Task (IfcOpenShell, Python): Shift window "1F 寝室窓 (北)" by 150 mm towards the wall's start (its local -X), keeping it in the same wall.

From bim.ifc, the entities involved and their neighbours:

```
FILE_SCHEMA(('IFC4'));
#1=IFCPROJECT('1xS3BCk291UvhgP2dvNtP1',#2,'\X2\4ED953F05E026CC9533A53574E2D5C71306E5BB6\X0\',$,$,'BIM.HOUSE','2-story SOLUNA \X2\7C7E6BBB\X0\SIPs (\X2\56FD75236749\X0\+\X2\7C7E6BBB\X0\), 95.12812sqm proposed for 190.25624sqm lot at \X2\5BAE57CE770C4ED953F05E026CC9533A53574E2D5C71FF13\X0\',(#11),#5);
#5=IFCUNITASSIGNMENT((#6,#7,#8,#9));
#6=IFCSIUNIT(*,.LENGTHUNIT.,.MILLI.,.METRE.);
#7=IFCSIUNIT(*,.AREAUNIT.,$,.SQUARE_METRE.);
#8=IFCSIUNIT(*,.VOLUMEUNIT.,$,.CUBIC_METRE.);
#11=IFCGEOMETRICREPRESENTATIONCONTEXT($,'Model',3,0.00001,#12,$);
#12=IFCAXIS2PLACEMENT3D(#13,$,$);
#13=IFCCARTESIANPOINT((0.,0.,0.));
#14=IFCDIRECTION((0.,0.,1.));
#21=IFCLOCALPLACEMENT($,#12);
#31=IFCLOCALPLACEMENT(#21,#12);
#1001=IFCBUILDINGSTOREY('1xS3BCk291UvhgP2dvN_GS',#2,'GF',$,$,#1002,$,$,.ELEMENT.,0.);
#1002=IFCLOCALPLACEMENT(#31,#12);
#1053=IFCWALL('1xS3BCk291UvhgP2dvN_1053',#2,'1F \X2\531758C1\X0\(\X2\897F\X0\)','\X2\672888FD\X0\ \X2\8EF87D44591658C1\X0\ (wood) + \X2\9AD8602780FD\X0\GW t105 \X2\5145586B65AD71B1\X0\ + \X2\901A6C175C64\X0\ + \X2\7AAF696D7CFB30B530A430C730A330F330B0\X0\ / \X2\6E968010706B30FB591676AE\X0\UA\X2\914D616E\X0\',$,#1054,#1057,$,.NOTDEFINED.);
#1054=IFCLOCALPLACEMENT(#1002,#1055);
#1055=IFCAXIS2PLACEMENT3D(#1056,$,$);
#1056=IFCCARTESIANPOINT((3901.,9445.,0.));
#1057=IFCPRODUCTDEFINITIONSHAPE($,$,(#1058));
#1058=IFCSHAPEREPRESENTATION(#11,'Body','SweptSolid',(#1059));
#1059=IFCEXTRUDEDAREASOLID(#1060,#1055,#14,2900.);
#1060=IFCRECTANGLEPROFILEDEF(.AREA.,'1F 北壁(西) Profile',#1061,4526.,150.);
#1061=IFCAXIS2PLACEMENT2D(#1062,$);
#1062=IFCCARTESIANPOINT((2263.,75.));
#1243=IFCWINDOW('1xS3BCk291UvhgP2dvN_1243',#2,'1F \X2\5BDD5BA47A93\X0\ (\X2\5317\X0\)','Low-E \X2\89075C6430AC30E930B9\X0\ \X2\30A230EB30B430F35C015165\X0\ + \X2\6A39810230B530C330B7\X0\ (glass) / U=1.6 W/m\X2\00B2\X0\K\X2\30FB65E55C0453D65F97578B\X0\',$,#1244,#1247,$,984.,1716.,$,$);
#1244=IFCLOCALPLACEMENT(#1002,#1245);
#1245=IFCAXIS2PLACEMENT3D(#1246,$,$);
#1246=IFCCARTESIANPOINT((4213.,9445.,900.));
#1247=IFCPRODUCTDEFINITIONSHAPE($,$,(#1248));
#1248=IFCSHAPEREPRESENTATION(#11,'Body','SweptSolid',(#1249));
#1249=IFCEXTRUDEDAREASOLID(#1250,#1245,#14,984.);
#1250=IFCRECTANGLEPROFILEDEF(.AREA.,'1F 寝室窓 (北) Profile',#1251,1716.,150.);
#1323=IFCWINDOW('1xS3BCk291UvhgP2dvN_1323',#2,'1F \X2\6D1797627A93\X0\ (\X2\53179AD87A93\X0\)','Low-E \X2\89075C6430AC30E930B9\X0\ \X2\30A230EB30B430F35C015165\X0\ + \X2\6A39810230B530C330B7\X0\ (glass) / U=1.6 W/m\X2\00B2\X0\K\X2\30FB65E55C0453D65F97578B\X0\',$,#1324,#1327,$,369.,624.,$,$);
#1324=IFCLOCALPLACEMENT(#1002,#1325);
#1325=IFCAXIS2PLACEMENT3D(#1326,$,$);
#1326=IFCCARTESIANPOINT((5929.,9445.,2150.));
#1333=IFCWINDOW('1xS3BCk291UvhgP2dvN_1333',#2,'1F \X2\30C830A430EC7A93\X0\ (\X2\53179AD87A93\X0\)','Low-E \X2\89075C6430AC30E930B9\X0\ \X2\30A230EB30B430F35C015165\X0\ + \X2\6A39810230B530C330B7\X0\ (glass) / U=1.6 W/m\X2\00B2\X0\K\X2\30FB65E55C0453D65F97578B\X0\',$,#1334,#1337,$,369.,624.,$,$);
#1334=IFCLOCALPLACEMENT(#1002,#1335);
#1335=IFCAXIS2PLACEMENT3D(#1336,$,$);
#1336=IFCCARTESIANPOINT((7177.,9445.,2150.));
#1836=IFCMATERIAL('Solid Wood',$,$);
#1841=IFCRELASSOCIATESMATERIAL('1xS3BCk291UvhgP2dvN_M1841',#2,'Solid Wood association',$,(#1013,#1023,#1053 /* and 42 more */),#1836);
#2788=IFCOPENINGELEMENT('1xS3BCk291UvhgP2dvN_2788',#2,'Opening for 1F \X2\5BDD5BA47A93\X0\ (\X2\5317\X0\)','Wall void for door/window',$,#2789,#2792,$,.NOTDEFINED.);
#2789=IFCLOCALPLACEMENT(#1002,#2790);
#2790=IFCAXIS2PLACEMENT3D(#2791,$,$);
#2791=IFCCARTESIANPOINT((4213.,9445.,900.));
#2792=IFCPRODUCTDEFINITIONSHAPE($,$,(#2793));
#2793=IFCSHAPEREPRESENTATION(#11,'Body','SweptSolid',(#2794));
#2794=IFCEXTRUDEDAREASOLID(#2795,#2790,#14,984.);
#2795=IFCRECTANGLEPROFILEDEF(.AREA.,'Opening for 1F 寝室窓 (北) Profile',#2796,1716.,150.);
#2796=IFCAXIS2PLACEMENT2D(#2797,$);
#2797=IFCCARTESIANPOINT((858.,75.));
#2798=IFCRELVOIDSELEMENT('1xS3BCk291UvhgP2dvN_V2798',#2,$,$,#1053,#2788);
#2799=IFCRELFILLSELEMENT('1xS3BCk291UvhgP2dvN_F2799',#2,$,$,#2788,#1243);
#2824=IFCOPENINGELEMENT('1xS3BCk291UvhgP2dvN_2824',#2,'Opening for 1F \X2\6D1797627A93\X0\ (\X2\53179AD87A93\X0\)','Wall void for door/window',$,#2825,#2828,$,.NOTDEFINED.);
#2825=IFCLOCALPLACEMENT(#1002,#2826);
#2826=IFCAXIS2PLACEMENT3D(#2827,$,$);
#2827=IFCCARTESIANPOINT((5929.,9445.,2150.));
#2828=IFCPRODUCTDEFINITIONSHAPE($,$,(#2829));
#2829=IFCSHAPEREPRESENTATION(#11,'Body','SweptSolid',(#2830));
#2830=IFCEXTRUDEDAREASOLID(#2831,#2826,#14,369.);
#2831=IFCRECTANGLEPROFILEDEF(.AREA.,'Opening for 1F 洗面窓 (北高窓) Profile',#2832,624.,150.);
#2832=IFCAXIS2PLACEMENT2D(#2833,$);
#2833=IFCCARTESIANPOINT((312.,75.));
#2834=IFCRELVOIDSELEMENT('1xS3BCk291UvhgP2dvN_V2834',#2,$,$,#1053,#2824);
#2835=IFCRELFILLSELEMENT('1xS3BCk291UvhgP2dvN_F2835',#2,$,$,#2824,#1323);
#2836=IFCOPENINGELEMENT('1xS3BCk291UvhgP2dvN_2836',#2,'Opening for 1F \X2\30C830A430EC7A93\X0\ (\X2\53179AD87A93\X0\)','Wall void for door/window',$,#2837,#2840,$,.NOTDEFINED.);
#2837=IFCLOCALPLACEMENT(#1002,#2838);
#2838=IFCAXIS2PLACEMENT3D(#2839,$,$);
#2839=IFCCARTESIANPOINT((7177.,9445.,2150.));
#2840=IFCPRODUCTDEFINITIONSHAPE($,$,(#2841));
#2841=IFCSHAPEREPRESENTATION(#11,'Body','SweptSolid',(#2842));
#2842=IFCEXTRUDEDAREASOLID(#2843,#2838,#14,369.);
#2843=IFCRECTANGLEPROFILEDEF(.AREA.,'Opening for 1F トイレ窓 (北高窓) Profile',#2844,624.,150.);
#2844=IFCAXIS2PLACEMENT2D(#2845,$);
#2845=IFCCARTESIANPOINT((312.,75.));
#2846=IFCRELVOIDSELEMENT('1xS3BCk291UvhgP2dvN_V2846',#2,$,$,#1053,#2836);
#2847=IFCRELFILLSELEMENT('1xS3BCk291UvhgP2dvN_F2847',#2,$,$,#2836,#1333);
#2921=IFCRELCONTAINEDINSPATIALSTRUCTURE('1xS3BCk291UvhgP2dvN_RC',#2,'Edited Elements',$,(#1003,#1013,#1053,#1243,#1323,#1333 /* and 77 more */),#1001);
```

```python
import ifcopenshell
import ifcopenshell.api.geometry
import ifcopenshell.util.placement
import ifcopenshell.util.unit

model = ifcopenshell.open("bim.ifc")
unit_scale = ifcopenshell.util.unit.calculate_unit_scale(model)

window = model.by_guid("1xS3BCk291UvhgP2dvN_1243")
opening = window.FillsVoids[0].RelatingOpeningElement
wall = opening.VoidsElements[0].RelatingBuildingElement

wall_matrix = ifcopenshell.util.placement.get_local_placement(wall.ObjectPlacement)
shift = wall_matrix[:3, 0] * -0.15 / unit_scale
before = ifcopenshell.util.placement.get_local_placement(window.ObjectPlacement)[:3, 3].copy()

# The window is not placed relative to its opening, so move both.
for product in (opening, window):
    matrix = ifcopenshell.util.placement.get_local_placement(product.ObjectPlacement)
    matrix[:3, 3] += shift
    ifcopenshell.api.geometry.edit_object_placement(model, product=product, matrix=matrix, is_si=False)

after = ifcopenshell.util.placement.get_local_placement(window.ObjectPlacement)[:3, 3]
print("window moved by", (after - before).round(3) + 0.0)

model.write("bim_updated.ifc")
```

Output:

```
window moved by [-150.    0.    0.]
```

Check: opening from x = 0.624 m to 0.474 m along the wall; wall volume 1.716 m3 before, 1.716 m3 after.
